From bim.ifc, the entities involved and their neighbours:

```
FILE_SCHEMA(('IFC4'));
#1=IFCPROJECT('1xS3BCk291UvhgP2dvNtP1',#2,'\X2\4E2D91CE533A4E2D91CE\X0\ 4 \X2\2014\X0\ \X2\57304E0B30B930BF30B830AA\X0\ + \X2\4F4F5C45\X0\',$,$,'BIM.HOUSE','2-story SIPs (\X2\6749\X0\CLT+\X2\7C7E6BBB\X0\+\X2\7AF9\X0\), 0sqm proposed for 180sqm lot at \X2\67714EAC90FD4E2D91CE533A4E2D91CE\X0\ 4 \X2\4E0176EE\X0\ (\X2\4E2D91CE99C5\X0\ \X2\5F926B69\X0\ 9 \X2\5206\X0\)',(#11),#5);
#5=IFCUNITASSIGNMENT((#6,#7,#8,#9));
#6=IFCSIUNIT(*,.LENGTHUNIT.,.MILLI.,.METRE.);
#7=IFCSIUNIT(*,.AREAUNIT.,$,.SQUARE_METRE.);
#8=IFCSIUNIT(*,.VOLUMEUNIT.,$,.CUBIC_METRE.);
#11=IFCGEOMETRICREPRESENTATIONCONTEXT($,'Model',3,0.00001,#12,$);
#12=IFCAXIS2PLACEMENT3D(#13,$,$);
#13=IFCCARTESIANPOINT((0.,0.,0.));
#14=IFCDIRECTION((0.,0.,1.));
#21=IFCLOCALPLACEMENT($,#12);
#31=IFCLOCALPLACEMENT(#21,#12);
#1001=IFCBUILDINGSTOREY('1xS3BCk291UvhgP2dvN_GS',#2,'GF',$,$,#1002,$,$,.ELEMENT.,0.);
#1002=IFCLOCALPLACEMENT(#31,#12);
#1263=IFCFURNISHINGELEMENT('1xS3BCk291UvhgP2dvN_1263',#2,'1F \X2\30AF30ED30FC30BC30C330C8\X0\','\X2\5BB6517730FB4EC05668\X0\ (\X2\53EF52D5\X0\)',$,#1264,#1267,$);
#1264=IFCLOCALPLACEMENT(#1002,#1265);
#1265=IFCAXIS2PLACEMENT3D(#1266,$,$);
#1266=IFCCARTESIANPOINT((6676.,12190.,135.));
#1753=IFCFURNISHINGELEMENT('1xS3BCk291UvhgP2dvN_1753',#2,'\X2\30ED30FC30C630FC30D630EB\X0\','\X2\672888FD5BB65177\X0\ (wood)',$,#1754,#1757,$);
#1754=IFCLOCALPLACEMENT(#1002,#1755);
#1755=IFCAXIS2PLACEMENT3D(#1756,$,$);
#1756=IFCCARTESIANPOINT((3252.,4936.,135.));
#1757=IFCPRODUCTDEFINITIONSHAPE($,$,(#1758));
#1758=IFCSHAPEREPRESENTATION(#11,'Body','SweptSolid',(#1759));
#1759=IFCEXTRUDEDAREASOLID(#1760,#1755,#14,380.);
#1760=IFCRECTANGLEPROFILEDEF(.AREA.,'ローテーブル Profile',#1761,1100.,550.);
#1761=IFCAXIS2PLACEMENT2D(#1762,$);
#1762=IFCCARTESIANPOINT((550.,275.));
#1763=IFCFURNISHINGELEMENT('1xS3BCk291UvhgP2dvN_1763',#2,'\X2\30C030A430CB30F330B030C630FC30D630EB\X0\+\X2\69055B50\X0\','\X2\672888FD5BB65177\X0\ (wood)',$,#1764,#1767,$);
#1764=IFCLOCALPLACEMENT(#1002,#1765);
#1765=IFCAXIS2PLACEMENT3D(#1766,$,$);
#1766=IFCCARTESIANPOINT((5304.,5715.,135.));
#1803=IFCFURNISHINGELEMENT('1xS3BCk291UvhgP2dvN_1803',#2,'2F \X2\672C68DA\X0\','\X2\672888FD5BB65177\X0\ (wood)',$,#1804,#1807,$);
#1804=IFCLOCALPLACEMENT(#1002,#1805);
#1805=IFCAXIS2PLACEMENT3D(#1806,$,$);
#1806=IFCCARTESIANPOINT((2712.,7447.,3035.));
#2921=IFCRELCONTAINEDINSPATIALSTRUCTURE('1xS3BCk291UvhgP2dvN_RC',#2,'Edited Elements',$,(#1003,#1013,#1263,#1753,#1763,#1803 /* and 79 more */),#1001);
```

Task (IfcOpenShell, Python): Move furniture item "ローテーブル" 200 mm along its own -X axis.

```python
import ifcopenshell
import ifcopenshell.api.geometry
import ifcopenshell.util.placement

model = ifcopenshell.open("bim.ifc")

item = model.by_guid("1xS3BCk291UvhgP2dvN_1753")
matrix = ifcopenshell.util.placement.get_local_placement(item.ObjectPlacement)
matrix[:3, 3] -= matrix[:3, 0] * 200.0
ifcopenshell.api.geometry.edit_object_placement(model, product=item, matrix=matrix, is_si=False)

print(ifcopenshell.util.placement.get_local_placement(item.ObjectPlacement).round(3) + 0.0)

model.write("bim_v2.ifc")
```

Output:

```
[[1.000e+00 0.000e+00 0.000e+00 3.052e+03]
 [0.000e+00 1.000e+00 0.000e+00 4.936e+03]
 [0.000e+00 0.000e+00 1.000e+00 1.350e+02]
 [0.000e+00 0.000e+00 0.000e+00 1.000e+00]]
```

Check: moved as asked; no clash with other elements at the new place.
